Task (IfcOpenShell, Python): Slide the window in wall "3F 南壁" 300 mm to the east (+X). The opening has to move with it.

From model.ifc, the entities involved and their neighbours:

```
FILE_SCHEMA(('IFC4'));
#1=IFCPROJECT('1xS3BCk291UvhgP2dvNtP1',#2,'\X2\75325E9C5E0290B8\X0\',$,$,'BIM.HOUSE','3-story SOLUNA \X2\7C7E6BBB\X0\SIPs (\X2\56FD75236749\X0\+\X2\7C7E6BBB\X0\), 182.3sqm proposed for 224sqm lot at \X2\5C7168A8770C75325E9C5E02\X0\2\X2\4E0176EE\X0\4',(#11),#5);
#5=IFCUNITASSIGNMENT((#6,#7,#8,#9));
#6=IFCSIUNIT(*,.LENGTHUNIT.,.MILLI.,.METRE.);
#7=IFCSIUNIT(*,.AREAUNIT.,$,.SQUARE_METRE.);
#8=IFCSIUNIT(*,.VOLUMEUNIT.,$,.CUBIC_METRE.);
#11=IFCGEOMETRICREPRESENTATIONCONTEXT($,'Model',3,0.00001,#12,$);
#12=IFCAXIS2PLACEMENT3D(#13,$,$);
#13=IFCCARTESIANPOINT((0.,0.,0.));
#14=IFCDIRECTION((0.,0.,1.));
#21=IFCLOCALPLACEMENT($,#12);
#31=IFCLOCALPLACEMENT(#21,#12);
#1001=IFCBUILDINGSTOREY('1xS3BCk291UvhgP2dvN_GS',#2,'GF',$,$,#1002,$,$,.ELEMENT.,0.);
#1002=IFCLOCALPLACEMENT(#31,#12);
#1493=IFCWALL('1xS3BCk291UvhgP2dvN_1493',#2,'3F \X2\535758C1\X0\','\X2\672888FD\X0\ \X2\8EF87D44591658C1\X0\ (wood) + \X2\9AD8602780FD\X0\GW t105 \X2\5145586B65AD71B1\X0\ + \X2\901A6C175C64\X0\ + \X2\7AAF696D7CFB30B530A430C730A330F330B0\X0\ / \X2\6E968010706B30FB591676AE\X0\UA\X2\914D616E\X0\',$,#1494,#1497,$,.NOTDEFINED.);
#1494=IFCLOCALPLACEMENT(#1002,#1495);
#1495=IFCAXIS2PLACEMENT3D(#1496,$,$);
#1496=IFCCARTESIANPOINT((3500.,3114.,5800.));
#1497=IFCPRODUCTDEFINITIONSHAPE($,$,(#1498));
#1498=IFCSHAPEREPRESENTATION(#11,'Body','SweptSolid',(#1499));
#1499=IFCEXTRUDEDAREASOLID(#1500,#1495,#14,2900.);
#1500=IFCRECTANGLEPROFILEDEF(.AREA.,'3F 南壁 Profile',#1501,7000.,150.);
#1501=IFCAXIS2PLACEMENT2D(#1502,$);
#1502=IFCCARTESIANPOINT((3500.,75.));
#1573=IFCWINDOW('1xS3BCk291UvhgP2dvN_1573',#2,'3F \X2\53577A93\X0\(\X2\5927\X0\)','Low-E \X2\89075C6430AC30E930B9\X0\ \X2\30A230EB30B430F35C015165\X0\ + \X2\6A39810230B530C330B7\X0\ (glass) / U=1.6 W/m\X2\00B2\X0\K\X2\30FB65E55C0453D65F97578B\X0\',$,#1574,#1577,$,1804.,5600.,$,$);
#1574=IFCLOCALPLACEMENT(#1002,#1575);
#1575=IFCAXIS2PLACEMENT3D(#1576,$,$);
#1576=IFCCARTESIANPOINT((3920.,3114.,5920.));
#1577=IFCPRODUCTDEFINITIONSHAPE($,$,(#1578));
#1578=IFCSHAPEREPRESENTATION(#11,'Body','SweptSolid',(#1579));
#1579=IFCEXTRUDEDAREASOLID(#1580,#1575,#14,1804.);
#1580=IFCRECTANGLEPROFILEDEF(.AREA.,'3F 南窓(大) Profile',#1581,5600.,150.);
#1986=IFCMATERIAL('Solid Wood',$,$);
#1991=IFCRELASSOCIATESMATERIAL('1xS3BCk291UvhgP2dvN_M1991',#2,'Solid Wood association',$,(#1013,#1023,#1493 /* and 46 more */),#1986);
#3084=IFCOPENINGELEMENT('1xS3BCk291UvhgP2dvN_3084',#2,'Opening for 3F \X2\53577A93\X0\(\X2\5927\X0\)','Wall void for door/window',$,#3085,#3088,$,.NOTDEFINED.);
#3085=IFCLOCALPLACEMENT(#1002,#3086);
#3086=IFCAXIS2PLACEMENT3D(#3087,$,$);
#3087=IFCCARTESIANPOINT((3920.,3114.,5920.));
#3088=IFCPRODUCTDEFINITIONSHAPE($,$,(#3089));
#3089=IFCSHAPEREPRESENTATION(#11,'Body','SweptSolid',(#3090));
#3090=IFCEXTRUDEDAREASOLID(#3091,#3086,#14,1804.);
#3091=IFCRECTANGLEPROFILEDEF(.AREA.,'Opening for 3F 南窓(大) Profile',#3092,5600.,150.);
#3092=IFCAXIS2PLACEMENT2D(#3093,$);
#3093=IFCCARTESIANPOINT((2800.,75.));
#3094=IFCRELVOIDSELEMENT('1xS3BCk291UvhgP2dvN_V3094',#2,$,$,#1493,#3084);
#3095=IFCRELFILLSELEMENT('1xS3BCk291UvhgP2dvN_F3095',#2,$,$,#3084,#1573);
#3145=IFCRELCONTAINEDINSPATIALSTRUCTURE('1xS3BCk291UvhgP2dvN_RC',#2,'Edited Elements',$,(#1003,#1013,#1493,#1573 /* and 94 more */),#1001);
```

```python
import ifcopenshell
import ifcopenshell.api.geometry
import ifcopenshell.util.placement

model = ifcopenshell.open("model.ifc")

window = model.by_id(1573)
opening = window.FillsVoids[0].RelatingOpeningElement
wall = opening.VoidsElements[0].RelatingBuildingElement

wall_matrix = ifcopenshell.util.placement.get_local_placement(wall.ObjectPlacement)
shift = wall_matrix[:3, 0] * 300.0
before = ifcopenshell.util.placement.get_local_placement(window.ObjectPlacement)[:3, 3].copy()

# The window is not placed relative to its opening, so move both.
for product in (opening, window):
    matrix = ifcopenshell.util.placement.get_local_placement(product.ObjectPlacement)
    matrix[:3, 3] += shift
    ifcopenshell.api.geometry.edit_object_placement(model, product=product, matrix=matrix, is_si=False)

after = ifcopenshell.util.placement.get_local_placement(window.ObjectPlacement)[:3, 3]
print("window moved by", (after - before).round(3) + 0.0)

model.write("model_v2.ifc")
```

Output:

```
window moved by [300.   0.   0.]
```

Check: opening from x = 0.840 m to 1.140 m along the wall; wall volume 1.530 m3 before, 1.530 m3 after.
